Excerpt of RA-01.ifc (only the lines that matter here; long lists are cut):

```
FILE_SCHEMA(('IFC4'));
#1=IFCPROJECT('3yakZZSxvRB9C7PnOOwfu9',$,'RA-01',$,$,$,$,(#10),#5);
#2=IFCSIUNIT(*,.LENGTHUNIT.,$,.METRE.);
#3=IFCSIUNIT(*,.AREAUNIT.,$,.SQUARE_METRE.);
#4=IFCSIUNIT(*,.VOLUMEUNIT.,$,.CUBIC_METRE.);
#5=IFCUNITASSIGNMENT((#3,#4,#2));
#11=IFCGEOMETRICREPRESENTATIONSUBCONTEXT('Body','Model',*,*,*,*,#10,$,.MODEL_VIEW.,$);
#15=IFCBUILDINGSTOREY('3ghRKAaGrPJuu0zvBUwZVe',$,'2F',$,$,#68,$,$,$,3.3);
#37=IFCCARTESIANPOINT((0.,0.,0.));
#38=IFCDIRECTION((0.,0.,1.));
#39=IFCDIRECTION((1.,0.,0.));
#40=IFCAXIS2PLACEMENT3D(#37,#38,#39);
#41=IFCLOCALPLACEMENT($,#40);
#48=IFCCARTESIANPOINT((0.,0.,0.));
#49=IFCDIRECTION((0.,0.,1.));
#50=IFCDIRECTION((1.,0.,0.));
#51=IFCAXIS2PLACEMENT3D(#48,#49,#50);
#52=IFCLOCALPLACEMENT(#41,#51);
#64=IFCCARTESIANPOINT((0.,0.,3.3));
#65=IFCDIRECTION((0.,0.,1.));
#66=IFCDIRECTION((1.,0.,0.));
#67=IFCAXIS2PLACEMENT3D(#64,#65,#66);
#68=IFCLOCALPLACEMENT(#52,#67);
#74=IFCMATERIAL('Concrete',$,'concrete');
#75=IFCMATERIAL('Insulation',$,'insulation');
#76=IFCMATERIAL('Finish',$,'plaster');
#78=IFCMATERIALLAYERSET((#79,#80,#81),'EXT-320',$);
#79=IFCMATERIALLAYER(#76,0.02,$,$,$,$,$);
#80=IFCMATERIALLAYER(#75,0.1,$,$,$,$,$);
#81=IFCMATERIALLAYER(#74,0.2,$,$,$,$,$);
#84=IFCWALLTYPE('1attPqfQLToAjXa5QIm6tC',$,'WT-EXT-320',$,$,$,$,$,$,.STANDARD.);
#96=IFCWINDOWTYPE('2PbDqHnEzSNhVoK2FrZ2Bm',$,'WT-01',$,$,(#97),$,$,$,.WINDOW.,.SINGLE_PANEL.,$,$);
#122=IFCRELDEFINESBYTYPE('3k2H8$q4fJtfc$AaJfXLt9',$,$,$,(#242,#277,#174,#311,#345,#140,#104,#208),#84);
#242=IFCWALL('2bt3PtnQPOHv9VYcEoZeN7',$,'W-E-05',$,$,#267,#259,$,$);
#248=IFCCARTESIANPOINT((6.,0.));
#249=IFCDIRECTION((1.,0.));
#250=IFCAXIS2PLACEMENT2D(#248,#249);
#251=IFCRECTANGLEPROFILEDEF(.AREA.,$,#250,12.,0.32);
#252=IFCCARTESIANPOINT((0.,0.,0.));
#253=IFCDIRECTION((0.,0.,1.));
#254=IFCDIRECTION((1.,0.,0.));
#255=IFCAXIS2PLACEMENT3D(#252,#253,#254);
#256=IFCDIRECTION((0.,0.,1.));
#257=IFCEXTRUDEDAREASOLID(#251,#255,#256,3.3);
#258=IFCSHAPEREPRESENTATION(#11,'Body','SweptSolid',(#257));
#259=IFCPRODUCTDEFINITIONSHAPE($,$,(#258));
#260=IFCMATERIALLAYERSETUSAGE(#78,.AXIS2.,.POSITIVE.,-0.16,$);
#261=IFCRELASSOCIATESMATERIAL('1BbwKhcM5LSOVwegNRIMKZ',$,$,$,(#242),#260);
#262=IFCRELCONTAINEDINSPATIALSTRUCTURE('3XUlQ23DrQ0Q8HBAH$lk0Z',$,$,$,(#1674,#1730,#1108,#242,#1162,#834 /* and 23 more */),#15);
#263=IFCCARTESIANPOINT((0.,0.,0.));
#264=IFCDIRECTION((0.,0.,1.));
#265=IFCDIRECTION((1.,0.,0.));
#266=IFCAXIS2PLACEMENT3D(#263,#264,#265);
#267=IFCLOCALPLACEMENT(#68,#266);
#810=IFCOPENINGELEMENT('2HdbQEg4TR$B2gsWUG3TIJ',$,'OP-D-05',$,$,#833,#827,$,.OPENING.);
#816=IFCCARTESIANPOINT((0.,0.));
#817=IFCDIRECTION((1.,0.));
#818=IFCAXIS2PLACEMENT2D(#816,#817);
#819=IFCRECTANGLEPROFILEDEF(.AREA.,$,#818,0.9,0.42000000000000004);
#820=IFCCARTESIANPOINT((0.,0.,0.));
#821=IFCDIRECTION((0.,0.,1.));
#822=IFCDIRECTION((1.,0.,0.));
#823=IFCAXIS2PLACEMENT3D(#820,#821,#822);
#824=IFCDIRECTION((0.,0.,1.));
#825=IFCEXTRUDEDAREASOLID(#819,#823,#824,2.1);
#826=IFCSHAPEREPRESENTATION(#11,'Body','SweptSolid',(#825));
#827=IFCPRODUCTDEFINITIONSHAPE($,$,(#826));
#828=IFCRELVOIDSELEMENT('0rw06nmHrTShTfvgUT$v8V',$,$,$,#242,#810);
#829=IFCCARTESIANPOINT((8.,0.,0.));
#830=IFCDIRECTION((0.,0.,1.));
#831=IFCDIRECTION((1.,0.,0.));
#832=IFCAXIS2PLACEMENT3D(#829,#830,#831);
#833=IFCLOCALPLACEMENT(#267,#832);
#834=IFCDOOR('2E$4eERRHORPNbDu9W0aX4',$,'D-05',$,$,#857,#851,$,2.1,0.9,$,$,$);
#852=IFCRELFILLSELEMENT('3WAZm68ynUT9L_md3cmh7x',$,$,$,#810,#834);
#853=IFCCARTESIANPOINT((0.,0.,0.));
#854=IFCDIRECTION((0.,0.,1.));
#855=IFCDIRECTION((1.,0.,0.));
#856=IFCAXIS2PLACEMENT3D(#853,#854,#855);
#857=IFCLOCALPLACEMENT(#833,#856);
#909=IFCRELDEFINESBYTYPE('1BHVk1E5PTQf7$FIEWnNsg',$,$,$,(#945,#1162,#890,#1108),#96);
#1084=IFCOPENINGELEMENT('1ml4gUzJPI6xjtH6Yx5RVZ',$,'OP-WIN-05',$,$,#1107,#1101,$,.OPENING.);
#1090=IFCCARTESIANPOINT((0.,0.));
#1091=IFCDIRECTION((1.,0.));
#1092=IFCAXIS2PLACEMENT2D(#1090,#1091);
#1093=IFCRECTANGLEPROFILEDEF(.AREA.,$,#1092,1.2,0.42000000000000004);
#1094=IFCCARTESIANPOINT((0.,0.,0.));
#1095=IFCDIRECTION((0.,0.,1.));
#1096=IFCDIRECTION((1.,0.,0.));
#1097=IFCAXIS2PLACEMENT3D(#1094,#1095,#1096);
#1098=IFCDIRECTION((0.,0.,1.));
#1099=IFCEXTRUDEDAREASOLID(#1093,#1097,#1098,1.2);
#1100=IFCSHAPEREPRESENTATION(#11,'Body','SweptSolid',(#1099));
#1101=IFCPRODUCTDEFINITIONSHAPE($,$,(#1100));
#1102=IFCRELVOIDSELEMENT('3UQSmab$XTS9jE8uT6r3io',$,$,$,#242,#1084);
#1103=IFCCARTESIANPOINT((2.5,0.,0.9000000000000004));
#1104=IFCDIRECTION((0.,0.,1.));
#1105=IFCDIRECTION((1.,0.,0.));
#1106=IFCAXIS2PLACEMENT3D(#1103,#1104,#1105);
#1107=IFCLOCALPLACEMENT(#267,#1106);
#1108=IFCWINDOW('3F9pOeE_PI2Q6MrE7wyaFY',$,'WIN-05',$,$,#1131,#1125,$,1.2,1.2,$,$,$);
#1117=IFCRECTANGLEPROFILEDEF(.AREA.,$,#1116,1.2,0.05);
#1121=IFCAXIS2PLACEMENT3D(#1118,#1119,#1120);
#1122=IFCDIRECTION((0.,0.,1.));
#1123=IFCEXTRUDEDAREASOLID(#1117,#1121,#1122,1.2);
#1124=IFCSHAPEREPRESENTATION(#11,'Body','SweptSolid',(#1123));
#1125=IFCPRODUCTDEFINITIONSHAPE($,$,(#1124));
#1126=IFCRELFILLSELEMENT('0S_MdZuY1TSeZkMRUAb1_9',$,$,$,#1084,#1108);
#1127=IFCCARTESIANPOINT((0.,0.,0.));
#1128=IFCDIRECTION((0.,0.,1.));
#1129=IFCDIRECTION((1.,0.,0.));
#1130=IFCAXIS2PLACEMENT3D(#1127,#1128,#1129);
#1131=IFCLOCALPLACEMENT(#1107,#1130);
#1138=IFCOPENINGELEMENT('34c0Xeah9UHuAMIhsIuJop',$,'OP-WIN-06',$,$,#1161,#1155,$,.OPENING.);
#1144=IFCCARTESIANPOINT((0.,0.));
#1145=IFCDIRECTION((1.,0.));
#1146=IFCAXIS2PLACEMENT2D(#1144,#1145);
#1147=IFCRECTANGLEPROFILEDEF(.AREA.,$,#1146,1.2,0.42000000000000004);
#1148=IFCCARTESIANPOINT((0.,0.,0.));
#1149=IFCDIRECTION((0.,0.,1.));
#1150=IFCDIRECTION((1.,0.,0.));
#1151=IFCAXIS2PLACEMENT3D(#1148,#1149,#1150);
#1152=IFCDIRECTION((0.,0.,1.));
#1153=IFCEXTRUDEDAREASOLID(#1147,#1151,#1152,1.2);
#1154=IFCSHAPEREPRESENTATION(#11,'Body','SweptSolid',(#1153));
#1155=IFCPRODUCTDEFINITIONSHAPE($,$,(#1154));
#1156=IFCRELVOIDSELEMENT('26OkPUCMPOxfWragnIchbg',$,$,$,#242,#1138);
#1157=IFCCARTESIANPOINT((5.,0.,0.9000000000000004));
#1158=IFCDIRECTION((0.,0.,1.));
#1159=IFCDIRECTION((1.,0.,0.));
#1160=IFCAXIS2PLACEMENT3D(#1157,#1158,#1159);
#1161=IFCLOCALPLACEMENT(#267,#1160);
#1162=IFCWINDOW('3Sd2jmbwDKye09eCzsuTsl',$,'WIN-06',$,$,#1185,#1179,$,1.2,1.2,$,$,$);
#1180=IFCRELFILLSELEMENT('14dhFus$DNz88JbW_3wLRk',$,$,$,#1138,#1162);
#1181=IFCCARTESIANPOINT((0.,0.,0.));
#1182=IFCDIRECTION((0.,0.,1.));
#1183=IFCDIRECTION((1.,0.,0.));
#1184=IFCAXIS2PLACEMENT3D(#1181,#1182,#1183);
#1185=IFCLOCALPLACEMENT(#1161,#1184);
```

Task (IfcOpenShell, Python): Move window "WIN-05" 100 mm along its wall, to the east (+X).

```python
import ifcopenshell
import ifcopenshell.api.geometry
import ifcopenshell.util.placement

model = ifcopenshell.open("RA-01.ifc")

window = model.by_id(1108)
opening = window.FillsVoids[0].RelatingOpeningElement
wall = opening.VoidsElements[0].RelatingBuildingElement

wall_matrix = ifcopenshell.util.placement.get_local_placement(wall.ObjectPlacement)
shift = wall_matrix[:3, 0] * 0.1
before = ifcopenshell.util.placement.get_local_placement(window.ObjectPlacement)[:3, 3].copy()

# The window is placed relative to its opening, so it follows when the opening moves.
matrix = ifcopenshell.util.placement.get_local_placement(opening.ObjectPlacement)
matrix[:3, 3] += shift
ifcopenshell.api.geometry.edit_object_placement(
    model, product=opening, matrix=matrix, is_si=False, should_transform_children=True
)

after = ifcopenshell.util.placement.get_local_placement(window.ObjectPlacement)[:3, 3]
print("window moved by", (after - before).round(3) + 0.0)

model.write("RA-01_v2.ifc")
```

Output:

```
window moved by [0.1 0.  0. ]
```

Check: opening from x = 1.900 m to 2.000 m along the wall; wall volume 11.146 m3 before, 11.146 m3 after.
